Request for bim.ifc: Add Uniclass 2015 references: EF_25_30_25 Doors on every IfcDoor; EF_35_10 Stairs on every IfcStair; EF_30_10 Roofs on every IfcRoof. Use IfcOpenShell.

First a look at what the model holds.

```python
import ifcopenshell

model = ifcopenshell.open("bim.ifc")
print(model.schema)
print("classifications:", [c.Name for c in model.by_type("IfcClassification")])
for ifc_class in ("IfcDoor", "IfcRoof", "IfcStair", "IfcWall", "IfcWindow"):
    print(ifc_class, len(model.by_type(ifc_class)))
```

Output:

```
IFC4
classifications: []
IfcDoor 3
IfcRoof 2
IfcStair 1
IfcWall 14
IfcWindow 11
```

```python
import ifcopenshell
import ifcopenshell.api.classification

model = ifcopenshell.open("bim.ifc")

system = ifcopenshell.api.classification.add_classification(model, classification="Uniclass 2015")

codes = {
    "IfcDoor": ("EF_25_30_25", "Doors"),
    "IfcStair": ("EF_35_10", "Stairs"),
    "IfcRoof": ("EF_30_10", "Roofs"),
}
for ifc_class, (code, name) in codes.items():
    products = model.by_type(ifc_class)
    ifcopenshell.api.classification.add_reference(
        model, products=products, classification=system, identification=code, name=name
    )
    print(code, len(products))

model.write("bim_v2.ifc")
```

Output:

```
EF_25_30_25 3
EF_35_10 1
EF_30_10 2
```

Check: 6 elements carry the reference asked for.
